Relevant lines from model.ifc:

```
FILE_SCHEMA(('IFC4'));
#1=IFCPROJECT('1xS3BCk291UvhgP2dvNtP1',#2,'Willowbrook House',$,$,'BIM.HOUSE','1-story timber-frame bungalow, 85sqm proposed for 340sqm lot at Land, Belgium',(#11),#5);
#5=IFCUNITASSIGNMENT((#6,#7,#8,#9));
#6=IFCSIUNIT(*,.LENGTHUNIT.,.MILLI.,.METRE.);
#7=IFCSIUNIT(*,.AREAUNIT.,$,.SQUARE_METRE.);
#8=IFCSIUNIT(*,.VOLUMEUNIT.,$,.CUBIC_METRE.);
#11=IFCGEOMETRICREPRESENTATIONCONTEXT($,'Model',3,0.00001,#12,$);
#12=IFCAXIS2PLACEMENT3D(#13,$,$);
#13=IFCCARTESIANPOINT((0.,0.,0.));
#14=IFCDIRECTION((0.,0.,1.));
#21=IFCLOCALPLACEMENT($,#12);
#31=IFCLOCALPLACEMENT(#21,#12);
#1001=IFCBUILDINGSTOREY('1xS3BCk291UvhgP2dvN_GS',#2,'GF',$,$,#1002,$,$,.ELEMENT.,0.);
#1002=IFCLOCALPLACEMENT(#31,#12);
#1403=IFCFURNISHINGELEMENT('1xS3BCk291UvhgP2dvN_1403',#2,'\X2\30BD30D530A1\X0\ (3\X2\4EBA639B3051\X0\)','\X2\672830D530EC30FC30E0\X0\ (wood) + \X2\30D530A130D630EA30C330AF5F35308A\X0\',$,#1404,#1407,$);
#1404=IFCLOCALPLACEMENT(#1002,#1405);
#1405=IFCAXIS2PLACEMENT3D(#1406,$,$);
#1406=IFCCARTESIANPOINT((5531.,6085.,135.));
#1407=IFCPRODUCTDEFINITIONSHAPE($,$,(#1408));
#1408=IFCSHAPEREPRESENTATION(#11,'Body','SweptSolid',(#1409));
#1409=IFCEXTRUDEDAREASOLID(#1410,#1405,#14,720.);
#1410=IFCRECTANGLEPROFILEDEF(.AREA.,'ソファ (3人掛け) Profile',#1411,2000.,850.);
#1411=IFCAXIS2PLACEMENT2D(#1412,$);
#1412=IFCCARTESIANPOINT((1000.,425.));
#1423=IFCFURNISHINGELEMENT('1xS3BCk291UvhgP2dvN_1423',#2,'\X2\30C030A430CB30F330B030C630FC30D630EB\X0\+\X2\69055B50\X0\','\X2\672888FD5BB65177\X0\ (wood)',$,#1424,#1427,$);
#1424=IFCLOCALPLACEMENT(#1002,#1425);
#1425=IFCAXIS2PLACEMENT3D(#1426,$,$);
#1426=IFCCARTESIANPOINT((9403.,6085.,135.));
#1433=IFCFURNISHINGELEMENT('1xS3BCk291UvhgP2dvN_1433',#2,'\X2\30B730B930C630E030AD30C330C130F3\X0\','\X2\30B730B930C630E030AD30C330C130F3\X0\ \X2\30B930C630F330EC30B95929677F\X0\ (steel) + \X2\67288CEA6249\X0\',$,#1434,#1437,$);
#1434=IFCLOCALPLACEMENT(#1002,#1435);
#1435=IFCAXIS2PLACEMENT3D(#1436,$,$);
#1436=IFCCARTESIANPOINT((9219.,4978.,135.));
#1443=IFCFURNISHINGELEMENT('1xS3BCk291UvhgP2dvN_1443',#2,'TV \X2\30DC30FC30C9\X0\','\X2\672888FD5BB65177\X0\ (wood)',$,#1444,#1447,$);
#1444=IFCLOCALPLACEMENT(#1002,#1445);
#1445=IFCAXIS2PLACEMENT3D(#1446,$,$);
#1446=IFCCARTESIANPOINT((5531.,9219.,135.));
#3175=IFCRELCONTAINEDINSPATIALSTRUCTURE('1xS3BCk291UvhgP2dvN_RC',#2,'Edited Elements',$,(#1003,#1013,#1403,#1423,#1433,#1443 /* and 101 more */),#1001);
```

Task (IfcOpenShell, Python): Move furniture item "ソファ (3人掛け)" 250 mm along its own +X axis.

```python
import ifcopenshell
import ifcopenshell.api.geometry
import ifcopenshell.util.placement
import ifcopenshell.util.unit

model = ifcopenshell.open("model.ifc")
unit_scale = ifcopenshell.util.unit.calculate_unit_scale(model)

item = model.by_id(1403)
matrix = ifcopenshell.util.placement.get_local_placement(item.ObjectPlacement)
matrix[:3, 3] += matrix[:3, 0] * 0.25 / unit_scale
ifcopenshell.api.geometry.edit_object_placement(model, product=item, matrix=matrix, is_si=False)

print(ifcopenshell.util.placement.get_local_placement(item.ObjectPlacement).round(3) + 0.0)

model.write("model_v2.ifc")
```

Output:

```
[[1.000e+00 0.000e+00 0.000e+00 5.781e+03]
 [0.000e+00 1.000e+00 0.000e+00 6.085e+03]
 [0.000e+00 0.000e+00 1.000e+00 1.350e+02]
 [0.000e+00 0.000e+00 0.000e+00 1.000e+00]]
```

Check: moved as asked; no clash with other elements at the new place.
